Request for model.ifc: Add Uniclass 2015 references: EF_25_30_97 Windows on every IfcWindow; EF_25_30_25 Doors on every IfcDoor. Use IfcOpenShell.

First a look at what the model holds.

```python
import ifcopenshell

model = ifcopenshell.open("model.ifc")
print(model.schema)
print("classifications:", [c.Name for c in model.by_type("IfcClassification")])
for ifc_class in ("IfcDoor", "IfcRoof", "IfcStair", "IfcWall", "IfcWindow"):
    print(ifc_class, len(model.by_type(ifc_class)))
```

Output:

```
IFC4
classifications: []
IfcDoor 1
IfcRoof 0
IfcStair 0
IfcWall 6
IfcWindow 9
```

```python
import ifcopenshell
import ifcopenshell.api.classification

model = ifcopenshell.open("model.ifc")

system = ifcopenshell.api.classification.add_classification(model, classification="Uniclass 2015")

codes = {
    "IfcWindow": ("EF_25_30_97", "Windows"),
    "IfcDoor": ("EF_25_30_25", "Doors"),
}
for ifc_class, (code, name) in codes.items():
    products = model.by_type(ifc_class)
    ifcopenshell.api.classification.add_reference(
        model, products=products, classification=system, identification=code, name=name
    )
    print(code, len(products))

model.write("model_v2.ifc")
```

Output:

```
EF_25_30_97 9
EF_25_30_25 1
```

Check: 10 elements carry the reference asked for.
